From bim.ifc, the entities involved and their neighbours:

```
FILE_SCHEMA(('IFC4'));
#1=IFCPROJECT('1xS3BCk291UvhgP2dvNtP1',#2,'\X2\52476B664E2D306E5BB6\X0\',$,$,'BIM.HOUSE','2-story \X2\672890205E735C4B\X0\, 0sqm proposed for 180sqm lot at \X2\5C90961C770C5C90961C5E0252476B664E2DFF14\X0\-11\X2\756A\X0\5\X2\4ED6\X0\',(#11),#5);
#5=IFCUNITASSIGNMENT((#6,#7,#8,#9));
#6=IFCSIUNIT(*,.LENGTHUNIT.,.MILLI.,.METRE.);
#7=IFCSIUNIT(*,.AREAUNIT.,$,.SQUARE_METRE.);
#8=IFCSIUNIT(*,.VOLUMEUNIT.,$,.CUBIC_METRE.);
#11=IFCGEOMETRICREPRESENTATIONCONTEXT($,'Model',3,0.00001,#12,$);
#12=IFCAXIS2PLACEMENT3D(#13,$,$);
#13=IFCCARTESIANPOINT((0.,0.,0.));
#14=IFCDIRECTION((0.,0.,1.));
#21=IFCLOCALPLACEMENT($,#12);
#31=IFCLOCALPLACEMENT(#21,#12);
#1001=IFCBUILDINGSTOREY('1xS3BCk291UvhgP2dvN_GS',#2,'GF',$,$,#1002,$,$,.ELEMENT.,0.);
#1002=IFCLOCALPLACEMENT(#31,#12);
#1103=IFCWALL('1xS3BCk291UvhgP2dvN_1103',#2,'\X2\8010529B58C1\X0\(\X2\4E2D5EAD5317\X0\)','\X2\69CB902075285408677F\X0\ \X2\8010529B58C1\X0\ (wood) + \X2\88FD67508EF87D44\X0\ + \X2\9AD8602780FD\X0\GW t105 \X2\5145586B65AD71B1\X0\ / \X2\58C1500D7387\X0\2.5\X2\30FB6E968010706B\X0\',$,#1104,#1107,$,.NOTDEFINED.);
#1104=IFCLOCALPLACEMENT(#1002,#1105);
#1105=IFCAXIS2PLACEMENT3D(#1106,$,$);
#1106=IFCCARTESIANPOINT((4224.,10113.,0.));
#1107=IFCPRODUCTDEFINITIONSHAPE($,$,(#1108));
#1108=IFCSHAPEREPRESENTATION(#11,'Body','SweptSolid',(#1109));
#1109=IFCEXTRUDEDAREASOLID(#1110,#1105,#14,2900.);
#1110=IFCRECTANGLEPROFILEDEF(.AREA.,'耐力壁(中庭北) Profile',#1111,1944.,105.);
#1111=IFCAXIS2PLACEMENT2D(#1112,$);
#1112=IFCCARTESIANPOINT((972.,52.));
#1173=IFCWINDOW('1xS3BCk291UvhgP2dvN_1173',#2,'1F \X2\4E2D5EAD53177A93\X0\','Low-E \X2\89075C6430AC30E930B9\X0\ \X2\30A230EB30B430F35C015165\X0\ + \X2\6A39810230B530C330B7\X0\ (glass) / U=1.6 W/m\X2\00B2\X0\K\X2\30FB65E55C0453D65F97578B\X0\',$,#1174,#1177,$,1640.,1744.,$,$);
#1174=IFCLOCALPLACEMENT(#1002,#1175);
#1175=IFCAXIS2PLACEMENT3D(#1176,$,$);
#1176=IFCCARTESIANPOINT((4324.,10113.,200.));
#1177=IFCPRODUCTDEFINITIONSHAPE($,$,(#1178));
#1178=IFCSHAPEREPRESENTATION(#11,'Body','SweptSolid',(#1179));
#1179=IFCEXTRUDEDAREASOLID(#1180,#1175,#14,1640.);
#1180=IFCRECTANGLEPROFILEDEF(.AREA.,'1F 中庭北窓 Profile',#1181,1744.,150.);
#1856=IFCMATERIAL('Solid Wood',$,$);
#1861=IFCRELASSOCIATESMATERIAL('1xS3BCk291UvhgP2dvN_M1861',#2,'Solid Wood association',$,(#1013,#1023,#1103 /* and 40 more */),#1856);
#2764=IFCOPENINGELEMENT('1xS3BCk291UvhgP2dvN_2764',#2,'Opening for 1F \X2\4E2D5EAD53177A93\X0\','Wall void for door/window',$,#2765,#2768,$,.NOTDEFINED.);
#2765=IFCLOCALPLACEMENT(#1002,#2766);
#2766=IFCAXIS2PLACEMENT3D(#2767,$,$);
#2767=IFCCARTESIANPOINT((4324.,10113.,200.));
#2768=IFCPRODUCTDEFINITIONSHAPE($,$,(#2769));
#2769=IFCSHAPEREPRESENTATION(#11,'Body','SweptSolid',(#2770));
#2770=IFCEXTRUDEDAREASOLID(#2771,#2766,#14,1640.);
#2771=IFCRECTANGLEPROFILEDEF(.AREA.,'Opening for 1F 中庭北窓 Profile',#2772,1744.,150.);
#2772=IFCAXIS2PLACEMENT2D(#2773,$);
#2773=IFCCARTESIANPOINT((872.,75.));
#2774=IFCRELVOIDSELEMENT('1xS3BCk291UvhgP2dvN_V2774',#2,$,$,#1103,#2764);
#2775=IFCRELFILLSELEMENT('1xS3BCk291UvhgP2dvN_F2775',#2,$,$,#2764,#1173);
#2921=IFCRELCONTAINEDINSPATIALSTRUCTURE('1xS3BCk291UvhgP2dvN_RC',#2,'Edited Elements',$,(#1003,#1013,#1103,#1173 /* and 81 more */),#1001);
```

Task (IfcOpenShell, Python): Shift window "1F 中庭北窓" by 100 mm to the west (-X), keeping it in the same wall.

```python
import ifcopenshell
import ifcopenshell.api.geometry
import ifcopenshell.util.placement
import ifcopenshell.util.unit

model = ifcopenshell.open("bim.ifc")
unit_scale = ifcopenshell.util.unit.calculate_unit_scale(model)

window = model.by_guid("1xS3BCk291UvhgP2dvN_1173")
opening = window.FillsVoids[0].RelatingOpeningElement
wall = opening.VoidsElements[0].RelatingBuildingElement

wall_matrix = ifcopenshell.util.placement.get_local_placement(wall.ObjectPlacement)
shift = wall_matrix[:3, 0] * -0.1 / unit_scale
before = ifcopenshell.util.placement.get_local_placement(window.ObjectPlacement)[:3, 3].copy()

# The window is not placed relative to its opening, so move both.
for product in (opening, window):
    matrix = ifcopenshell.util.placement.get_local_placement(product.ObjectPlacement)
    matrix[:3, 3] += shift
    ifcopenshell.api.geometry.edit_object_placement(model, product=product, matrix=matrix, is_si=False)

after = ifcopenshell.util.placement.get_local_placement(window.ObjectPlacement)[:3, 3]
print("window moved by", (after - before).round(3) + 0.0)

model.write("bim_v2.ifc")
```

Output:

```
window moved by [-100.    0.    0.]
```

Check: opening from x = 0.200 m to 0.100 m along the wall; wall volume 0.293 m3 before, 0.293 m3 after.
